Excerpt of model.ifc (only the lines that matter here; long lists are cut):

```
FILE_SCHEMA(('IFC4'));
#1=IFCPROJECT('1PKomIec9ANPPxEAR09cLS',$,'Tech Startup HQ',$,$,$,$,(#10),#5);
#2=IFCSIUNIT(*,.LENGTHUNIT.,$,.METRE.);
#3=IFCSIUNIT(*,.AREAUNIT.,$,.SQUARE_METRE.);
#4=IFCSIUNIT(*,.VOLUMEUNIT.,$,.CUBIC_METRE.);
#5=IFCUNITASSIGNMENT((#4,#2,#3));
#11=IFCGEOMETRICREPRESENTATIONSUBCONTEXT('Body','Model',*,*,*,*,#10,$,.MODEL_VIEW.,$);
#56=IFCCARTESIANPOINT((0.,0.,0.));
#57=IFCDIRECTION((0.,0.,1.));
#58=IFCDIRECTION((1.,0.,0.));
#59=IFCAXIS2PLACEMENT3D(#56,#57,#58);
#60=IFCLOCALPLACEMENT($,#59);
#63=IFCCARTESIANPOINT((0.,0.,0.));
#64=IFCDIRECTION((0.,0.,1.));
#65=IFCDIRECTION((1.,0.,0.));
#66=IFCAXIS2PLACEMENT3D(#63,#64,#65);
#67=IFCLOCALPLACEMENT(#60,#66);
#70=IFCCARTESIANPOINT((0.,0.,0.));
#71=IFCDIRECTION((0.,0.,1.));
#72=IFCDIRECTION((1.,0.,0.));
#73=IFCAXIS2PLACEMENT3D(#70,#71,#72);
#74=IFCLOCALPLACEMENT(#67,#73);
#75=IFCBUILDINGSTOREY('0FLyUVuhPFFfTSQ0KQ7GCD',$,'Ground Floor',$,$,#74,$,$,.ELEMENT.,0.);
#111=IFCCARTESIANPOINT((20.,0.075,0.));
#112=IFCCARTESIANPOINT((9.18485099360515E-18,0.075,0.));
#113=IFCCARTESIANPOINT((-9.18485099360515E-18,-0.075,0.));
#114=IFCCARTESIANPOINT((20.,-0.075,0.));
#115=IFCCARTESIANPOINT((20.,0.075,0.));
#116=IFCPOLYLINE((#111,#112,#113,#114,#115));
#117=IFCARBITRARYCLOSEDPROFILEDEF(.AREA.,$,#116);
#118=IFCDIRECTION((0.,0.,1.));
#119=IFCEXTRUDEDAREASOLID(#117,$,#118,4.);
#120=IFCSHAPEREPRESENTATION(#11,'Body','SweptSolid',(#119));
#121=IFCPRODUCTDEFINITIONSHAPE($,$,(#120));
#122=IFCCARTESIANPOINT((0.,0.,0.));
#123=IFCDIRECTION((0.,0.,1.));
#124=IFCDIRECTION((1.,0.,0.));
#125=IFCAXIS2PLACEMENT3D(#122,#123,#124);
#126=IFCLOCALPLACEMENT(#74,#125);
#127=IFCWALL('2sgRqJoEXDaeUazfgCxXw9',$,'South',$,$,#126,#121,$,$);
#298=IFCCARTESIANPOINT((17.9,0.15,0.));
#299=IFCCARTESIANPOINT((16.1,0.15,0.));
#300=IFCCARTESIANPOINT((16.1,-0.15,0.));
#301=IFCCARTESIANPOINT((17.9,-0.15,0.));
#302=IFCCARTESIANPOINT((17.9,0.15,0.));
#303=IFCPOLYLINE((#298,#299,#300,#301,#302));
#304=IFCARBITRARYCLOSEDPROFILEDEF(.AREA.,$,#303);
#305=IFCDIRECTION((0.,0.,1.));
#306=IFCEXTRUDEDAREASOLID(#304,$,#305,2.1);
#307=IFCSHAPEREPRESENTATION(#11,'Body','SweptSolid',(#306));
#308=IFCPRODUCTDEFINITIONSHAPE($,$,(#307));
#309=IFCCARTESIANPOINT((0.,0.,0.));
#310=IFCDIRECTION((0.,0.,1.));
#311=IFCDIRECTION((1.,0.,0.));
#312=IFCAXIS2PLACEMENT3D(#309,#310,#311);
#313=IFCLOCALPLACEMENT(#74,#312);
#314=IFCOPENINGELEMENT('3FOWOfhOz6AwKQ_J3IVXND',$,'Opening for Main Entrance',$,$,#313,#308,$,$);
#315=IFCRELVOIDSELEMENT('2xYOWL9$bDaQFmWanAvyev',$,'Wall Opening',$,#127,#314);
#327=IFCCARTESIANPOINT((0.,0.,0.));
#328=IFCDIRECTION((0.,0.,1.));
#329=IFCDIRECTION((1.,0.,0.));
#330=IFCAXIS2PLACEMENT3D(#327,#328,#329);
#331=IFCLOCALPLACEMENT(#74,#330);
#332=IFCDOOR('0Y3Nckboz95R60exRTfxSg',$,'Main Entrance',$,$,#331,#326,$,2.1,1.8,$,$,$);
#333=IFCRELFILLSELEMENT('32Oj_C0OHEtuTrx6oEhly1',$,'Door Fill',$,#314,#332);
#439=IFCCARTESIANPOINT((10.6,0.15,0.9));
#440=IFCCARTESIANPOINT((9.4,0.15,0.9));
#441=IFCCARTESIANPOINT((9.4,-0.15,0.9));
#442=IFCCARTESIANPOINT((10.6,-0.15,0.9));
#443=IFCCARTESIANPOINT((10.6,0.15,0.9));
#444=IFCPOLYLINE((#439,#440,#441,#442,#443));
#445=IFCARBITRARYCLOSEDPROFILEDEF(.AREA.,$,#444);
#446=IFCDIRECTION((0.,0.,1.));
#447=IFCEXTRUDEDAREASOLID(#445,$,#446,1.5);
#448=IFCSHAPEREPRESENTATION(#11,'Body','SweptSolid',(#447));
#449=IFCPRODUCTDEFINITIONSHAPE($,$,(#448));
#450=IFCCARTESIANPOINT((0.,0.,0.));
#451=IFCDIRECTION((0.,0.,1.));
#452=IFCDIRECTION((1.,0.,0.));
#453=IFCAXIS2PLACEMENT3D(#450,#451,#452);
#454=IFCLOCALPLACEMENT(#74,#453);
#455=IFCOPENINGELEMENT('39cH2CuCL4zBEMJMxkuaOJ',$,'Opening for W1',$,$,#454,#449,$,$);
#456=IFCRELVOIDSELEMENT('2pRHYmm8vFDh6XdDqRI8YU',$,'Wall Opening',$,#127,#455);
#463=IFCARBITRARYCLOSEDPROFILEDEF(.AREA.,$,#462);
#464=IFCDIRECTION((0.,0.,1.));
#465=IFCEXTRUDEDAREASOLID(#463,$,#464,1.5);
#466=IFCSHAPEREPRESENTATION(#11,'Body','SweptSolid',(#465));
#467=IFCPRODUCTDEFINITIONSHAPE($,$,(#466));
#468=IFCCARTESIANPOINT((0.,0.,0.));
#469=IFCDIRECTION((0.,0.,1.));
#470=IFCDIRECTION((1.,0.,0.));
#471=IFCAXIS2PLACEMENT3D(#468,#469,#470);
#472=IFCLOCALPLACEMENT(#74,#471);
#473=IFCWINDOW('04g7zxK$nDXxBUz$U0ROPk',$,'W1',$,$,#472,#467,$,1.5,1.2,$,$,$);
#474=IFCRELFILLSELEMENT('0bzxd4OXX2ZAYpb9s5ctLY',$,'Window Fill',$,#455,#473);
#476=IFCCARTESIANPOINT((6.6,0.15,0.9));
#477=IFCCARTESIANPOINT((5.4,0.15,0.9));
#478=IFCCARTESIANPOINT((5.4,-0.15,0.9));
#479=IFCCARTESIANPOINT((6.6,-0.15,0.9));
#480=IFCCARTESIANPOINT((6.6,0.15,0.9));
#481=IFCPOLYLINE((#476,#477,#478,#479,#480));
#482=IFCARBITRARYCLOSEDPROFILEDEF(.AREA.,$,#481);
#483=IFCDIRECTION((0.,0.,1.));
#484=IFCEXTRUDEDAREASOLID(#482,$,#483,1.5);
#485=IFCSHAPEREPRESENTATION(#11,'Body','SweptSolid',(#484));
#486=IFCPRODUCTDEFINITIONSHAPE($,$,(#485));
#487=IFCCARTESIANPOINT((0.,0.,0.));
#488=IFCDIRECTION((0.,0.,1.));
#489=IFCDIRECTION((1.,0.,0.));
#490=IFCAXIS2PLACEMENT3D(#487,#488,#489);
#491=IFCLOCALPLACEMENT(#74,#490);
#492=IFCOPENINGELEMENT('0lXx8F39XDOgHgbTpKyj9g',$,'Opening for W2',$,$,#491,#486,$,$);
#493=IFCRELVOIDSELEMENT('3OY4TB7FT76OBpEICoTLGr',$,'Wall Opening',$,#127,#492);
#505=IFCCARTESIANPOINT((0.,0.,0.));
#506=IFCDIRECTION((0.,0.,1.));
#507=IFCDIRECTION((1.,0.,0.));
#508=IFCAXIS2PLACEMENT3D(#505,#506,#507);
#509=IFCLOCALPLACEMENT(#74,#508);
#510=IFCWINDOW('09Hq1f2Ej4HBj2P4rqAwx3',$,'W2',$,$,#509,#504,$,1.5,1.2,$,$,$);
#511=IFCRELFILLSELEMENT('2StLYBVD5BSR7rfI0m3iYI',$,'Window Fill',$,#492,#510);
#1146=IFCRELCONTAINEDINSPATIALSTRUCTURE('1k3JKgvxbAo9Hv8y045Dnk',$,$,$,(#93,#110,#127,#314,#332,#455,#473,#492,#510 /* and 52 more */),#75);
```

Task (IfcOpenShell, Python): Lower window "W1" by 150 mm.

```python
import numpy as np
import ifcopenshell
import ifcopenshell.api.geometry
import ifcopenshell.util.placement
import ifcopenshell.util.unit

model = ifcopenshell.open("model.ifc")
unit_scale = ifcopenshell.util.unit.calculate_unit_scale(model)

window = model.by_guid("04g7zxK$nDXxBUz$U0ROPk")
opening = window.FillsVoids[0].RelatingOpeningElement
dz = -0.15 / unit_scale

shift = np.array([0.0, 0.0, dz])
# The window is not placed relative to its opening, so move both.
for product in (opening, window):
    matrix = ifcopenshell.util.placement.get_local_placement(product.ObjectPlacement)
    matrix[:3, 3] += shift
    ifcopenshell.api.geometry.edit_object_placement(model, product=product, matrix=matrix, is_si=False)

print(f"moved by {dz * unit_scale:+.3f} m")

model.write("model_updated.ifc")
```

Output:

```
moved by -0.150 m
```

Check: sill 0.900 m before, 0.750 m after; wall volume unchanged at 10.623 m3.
